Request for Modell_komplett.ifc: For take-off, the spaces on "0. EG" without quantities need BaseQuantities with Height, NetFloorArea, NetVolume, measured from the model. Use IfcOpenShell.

First a look at what the model holds.

```python
import ifcopenshell
import ifcopenshell.util.element
import ifcopenshell.util.unit

model = ifcopenshell.open("Modell_komplett.ifc")
print(model.schema)
for unit_type in ("LENGTHUNIT", "AREAUNIT", "VOLUMEUNIT"):
    print(unit_type, ifcopenshell.util.unit.calculate_unit_scale(model, unit_type))
storey = next(s for s in model.by_type("IfcBuildingStorey") if s.Name == "0. EG")
spaces = [e for e in ifcopenshell.util.element.get_decomposition(storey) if e.is_a("IfcSpace")]
for e in sorted(spaces, key=lambda e: e.id()):
    print(e.id(), e.is_a(), e.Name, list(ifcopenshell.util.element.get_psets(e, qtos_only=True)), sep=" | ")
```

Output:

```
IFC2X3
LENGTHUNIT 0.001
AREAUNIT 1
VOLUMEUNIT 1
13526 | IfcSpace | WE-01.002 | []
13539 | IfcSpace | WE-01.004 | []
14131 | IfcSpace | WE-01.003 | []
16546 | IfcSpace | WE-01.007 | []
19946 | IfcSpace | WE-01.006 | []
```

```python
import ifcopenshell
import ifcopenshell.api.pset
import ifcopenshell.geom
import ifcopenshell.util.element
import ifcopenshell.util.shape
import ifcopenshell.util.unit

model = ifcopenshell.open("Modell_komplett.ifc")
unit_scale = ifcopenshell.util.unit.calculate_unit_scale(model)
area_scale = ifcopenshell.util.unit.calculate_unit_scale(model, "AREAUNIT")
volume_scale = ifcopenshell.util.unit.calculate_unit_scale(model, "VOLUMEUNIT")
settings = ifcopenshell.geom.settings()

storey = next(s for s in model.by_type("IfcBuildingStorey") if s.Name == "0. EG")
spaces = [e for e in ifcopenshell.util.element.get_decomposition(storey) if e.is_a("IfcSpace")]

for e in sorted(spaces, key=lambda e: e.id()):
    if ifcopenshell.util.element.get_psets(e, qtos_only=True, should_inherit=False):
        continue
    # Geometry comes back in metres, in the element's own axes.
    shape = ifcopenshell.geom.create_shape(settings, e)
    values = {
        "Height": ifcopenshell.util.shape.get_z(shape.geometry) / unit_scale,
        "NetFloorArea": ifcopenshell.util.shape.get_footprint_area(shape.geometry) / area_scale,
        "NetVolume": ifcopenshell.util.shape.get_volume(shape.geometry) / volume_scale,
    }
    qto = ifcopenshell.api.pset.add_qto(model, product=e, name="BaseQuantities")
    ifcopenshell.api.pset.edit_qto(model, qto=qto, properties=values)
    print(e.id(), {k: round(v, 3) for k, v in values.items()})

model.write("Modell_komplett_updated.ifc")
```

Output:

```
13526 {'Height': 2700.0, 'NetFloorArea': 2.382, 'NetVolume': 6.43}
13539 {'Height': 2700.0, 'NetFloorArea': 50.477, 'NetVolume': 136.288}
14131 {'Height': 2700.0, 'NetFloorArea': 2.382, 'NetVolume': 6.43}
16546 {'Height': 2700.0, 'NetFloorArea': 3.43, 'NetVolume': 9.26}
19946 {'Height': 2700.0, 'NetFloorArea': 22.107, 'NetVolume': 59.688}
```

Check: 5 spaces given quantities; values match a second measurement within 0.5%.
